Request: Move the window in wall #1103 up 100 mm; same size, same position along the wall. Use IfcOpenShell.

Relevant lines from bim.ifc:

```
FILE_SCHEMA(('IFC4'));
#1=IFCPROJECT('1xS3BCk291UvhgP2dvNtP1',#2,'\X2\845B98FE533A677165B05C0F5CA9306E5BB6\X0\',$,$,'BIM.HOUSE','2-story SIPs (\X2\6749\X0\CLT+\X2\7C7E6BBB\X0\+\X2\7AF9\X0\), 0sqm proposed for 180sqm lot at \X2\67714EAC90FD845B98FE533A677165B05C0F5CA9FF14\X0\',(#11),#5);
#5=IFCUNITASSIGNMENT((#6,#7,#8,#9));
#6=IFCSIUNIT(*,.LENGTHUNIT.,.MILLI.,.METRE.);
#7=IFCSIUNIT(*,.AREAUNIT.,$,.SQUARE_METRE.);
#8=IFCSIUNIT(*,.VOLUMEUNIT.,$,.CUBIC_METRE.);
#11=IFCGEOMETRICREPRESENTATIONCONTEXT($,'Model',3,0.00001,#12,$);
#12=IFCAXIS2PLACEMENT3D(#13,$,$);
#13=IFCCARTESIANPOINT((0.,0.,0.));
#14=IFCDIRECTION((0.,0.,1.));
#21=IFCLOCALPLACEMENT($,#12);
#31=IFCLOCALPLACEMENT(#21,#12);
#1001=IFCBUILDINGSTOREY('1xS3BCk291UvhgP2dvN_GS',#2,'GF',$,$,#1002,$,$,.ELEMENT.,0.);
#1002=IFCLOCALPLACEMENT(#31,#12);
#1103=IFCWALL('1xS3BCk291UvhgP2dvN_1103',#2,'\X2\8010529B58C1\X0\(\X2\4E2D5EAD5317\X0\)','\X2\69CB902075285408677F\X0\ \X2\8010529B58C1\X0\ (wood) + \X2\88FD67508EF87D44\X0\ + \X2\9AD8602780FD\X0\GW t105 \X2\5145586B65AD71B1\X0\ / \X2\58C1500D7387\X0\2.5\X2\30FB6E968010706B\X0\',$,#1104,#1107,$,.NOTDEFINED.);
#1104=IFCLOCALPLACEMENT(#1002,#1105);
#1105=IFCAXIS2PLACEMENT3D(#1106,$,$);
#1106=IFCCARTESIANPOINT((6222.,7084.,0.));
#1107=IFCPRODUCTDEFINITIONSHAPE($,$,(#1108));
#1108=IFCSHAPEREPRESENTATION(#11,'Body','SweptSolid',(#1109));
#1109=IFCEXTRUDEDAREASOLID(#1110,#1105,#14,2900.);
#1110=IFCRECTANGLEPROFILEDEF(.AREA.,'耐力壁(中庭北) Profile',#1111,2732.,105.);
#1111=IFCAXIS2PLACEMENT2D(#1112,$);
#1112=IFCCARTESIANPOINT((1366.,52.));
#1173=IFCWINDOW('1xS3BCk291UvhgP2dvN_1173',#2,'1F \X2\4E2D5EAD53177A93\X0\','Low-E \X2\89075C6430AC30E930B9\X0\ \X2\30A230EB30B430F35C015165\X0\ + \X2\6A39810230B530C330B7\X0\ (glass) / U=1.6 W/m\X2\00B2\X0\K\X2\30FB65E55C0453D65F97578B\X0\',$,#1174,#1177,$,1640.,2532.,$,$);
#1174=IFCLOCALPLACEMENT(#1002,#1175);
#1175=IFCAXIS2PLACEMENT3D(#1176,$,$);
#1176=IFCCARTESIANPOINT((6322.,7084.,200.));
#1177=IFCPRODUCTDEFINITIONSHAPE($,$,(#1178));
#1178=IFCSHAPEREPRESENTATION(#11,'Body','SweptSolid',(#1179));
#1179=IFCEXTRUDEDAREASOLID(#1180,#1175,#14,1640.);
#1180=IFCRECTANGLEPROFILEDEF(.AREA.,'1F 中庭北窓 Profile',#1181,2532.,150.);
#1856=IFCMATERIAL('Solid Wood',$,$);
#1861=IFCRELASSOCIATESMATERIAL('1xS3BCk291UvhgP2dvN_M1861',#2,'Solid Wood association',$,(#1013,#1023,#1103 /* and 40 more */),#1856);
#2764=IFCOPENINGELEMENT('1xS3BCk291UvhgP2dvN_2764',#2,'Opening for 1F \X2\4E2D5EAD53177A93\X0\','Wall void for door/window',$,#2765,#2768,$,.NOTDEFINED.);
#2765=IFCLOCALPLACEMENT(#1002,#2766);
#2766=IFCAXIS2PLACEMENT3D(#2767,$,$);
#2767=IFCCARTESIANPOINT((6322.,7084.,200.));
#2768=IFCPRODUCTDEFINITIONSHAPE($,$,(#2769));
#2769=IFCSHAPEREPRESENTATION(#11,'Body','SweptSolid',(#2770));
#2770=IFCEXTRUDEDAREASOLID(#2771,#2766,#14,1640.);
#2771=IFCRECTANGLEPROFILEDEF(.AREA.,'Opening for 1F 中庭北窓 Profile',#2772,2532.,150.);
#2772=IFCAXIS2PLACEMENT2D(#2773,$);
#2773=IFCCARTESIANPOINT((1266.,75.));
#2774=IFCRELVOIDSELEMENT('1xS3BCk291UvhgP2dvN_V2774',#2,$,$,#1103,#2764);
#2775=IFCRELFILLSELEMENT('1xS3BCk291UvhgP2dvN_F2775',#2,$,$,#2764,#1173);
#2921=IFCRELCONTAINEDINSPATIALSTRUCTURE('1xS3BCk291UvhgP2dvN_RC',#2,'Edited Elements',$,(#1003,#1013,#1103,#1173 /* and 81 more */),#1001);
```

```python
import numpy as np
import ifcopenshell
import ifcopenshell.api.geometry
import ifcopenshell.util.placement
import ifcopenshell.util.unit

model = ifcopenshell.open("bim.ifc")
unit_scale = ifcopenshell.util.unit.calculate_unit_scale(model)

window = model.by_id(1173)
opening = window.FillsVoids[0].RelatingOpeningElement
dz = 100.0

shift = np.array([0.0, 0.0, dz])
# The window is not placed relative to its opening, so move both.
for product in (opening, window):
    matrix = ifcopenshell.util.placement.get_local_placement(product.ObjectPlacement)
    matrix[:3, 3] += shift
    ifcopenshell.api.geometry.edit_object_placement(model, product=product, matrix=matrix, is_si=False)

print(f"moved by {dz * unit_scale:+.3f} m")

model.write("bim_rev.ifc")
```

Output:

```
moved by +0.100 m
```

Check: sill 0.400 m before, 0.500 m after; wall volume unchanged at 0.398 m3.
